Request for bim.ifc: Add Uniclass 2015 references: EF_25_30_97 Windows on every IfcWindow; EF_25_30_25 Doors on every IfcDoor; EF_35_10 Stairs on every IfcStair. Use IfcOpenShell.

First a look at what the model holds.

```python
import ifcopenshell

model = ifcopenshell.open("bim.ifc")
print(model.schema)
print("classifications:", [c.Name for c in model.by_type("IfcClassification")])
for ifc_class in ("IfcDoor", "IfcRoof", "IfcStair", "IfcWall", "IfcWindow"):
    print(ifc_class, len(model.by_type(ifc_class)))
```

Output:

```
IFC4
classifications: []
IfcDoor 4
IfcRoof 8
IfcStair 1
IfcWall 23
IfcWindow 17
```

```python
import ifcopenshell
import ifcopenshell.api.classification

model = ifcopenshell.open("bim.ifc")

system = ifcopenshell.api.classification.add_classification(model, classification="Uniclass 2015")

codes = {
    "IfcWindow": ("EF_25_30_97", "Windows"),
    "IfcDoor": ("EF_25_30_25", "Doors"),
    "IfcStair": ("EF_35_10", "Stairs"),
}
for ifc_class, (code, name) in codes.items():
    products = model.by_type(ifc_class)
    ifcopenshell.api.classification.add_reference(
        model, products=products, classification=system, identification=code, name=name
    )
    print(code, len(products))

model.write("bim_v2.ifc")
```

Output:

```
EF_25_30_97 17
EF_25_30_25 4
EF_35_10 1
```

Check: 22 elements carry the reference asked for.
